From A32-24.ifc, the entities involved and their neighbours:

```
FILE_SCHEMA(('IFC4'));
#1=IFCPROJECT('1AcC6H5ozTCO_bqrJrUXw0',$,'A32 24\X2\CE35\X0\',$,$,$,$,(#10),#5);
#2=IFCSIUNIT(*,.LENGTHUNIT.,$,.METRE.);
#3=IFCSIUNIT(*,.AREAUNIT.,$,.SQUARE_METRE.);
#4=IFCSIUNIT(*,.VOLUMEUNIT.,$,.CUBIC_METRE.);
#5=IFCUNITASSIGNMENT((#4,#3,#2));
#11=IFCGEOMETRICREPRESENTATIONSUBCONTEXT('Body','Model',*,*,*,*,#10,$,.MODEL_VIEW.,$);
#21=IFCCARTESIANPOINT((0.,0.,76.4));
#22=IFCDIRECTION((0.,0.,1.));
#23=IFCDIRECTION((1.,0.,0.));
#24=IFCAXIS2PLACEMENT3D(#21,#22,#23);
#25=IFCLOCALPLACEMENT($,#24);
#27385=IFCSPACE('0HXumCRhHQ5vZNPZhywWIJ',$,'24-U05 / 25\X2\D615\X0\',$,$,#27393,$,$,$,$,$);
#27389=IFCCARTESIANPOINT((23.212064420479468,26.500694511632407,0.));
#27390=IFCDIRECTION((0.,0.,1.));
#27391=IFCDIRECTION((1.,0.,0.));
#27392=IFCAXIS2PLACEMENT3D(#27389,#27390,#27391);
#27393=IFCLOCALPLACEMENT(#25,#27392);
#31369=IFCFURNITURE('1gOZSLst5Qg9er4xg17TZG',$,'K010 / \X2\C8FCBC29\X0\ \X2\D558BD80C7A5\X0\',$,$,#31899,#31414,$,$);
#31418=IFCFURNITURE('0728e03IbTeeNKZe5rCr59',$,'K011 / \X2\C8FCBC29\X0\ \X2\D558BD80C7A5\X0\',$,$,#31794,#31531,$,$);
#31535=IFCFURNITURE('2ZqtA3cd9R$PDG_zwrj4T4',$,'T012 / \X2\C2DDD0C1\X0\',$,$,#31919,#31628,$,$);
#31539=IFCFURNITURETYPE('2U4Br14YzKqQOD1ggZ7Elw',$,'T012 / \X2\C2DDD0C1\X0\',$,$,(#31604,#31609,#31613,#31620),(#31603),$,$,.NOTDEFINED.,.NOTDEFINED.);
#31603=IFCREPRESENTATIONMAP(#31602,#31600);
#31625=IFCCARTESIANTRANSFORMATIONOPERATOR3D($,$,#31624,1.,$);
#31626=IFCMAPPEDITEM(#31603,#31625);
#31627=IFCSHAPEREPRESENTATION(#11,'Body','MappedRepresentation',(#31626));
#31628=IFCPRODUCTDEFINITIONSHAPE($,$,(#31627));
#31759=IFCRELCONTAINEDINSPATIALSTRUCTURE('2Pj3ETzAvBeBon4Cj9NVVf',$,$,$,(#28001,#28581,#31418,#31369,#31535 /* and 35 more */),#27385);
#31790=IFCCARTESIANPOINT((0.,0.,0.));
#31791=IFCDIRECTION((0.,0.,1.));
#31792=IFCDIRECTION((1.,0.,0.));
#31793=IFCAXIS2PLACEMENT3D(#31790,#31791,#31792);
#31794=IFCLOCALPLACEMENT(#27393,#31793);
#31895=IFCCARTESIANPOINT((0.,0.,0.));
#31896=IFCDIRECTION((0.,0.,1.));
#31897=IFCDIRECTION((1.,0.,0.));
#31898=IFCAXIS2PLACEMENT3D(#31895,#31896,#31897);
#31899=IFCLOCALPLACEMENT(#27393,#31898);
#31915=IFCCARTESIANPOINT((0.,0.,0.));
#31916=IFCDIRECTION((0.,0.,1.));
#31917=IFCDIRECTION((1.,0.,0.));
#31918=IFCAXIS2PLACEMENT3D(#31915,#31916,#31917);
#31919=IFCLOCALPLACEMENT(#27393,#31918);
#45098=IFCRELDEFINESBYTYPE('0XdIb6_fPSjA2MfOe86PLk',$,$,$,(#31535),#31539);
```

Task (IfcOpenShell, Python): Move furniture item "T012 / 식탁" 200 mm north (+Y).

```python
import ifcopenshell
import ifcopenshell.api.geometry
import ifcopenshell.util.placement
import ifcopenshell.util.unit

model = ifcopenshell.open("A32-24.ifc")
unit_scale = ifcopenshell.util.unit.calculate_unit_scale(model)

item = model.by_guid("2ZqtA3cd9R$PDG_zwrj4T4")
matrix = ifcopenshell.util.placement.get_local_placement(item.ObjectPlacement)
matrix[1, 3] += 0.2 / unit_scale
ifcopenshell.api.geometry.edit_object_placement(model, product=item, matrix=matrix, is_si=False)

print(ifcopenshell.util.placement.get_local_placement(item.ObjectPlacement).round(3) + 0.0)

model.write("A32-24_v2.ifc")
```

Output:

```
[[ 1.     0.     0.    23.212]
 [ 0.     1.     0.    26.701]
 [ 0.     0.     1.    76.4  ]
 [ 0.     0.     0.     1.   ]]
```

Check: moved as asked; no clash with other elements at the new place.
